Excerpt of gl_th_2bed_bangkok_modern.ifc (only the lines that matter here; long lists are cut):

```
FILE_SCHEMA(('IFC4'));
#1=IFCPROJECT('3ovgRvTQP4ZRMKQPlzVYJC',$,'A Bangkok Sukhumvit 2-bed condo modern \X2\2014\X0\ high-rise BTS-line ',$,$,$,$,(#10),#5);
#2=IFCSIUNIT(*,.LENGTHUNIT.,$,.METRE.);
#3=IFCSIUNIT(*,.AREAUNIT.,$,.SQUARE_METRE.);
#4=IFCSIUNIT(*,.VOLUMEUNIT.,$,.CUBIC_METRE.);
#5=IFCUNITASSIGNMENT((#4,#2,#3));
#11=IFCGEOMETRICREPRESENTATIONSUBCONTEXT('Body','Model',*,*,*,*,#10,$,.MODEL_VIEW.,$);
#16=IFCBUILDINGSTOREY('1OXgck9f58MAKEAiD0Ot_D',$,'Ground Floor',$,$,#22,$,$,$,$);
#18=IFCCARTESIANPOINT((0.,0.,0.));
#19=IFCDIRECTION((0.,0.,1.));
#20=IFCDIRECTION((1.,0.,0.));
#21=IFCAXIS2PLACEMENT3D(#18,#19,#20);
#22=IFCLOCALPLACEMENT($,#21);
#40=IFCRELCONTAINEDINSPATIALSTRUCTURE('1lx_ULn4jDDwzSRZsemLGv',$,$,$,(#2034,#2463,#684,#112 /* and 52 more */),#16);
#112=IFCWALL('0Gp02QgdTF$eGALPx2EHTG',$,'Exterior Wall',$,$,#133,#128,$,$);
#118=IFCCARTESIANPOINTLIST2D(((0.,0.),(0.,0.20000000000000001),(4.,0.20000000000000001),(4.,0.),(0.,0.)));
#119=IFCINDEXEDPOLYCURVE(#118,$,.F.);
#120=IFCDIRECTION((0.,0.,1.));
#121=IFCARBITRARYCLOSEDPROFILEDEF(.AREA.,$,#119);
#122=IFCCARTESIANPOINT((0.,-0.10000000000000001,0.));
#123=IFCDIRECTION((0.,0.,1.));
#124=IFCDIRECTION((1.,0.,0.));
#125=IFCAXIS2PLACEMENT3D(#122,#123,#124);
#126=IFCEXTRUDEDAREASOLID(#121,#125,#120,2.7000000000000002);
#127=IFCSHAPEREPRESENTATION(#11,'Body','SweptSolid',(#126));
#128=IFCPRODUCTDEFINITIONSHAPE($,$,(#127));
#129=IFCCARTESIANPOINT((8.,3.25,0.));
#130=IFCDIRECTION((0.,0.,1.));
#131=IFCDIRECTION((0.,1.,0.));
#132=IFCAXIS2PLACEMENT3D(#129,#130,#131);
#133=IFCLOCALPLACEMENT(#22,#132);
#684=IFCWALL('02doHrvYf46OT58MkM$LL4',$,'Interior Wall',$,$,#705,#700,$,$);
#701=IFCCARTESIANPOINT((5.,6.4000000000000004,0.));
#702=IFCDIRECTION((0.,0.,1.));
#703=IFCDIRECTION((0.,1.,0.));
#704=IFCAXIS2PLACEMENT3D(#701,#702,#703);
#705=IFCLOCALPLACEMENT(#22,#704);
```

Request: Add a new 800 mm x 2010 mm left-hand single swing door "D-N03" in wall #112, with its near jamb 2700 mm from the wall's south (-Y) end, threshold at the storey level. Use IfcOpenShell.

```python
import numpy as np
import ifcopenshell
import ifcopenshell.api.feature
import ifcopenshell.api.geometry
import ifcopenshell.api.root
import ifcopenshell.api.spatial
import ifcopenshell.geom
import ifcopenshell.util.element
import ifcopenshell.util.placement
import ifcopenshell.util.representation
import ifcopenshell.util.shape
import ifcopenshell.util.unit

model = ifcopenshell.open("gl_th_2bed_bangkok_modern.ifc")
unit_scale = ifcopenshell.util.unit.calculate_unit_scale(model)
settings = ifcopenshell.geom.settings()


def volume(element):
    """Net volume in cubic metres, openings subtracted."""
    shape = ifcopenshell.geom.create_shape(settings, element)
    return ifcopenshell.util.shape.get_volume(shape.geometry)


wall = model.by_guid("0Gp02QgdTF$eGALPx2EHTG")
storey = ifcopenshell.util.element.get_container(wall, ifc_class="IfcBuildingStorey")
context = ifcopenshell.util.representation.get_context(model, "Model", "Body", "MODEL_VIEW")
before = volume(wall)

width, height, from_end, sill = 0.8, 2.01, 2.7, 0.0  # metres

# The wall runs along its own X axis, and the end named is its -X end.
wall_shape = ifcopenshell.geom.create_shape(settings, wall)
x, y, z = ifcopenshell.util.shape.get_vertices(wall_shape.geometry).T
start = x.min() + from_end
face, thickness = float(y.min()), float(y.max() - y.min())
wall_matrix = ifcopenshell.util.placement.get_local_placement(wall.ObjectPlacement)
level = ifcopenshell.util.placement.get_local_placement(storey.ObjectPlacement)[2, 3]


def in_wall(x, y):
    """Placement at x, y metres in the wall's axes, at sill height."""
    matrix = wall_matrix.copy()
    matrix[:, 3] = wall_matrix @ np.array([x / unit_scale, y / unit_scale, 0.0, 1.0])
    matrix[2, 3] = level + sill / unit_scale
    return matrix


# Opening: a box that overshoots both wall faces by 50 mm.
opening = ifcopenshell.api.root.create_entity(model, ifc_class="IfcOpeningElement", predefined_type="OPENING")
box = ifcopenshell.api.geometry.add_wall_representation(
    model, context=context, length=width, height=height, thickness=thickness + 0.1
)
ifcopenshell.api.geometry.assign_representation(model, product=opening, representation=box)
ifcopenshell.api.geometry.edit_object_placement(model, product=opening, matrix=in_wall(start, face - 0.05), is_si=False)
ifcopenshell.api.feature.add_feature(model, feature=opening, element=wall)

door = ifcopenshell.api.root.create_entity(model, ifc_class="IfcDoor", name="D-N03", predefined_type="DOOR")
door.OverallWidth, door.OverallHeight = width / unit_scale, height / unit_scale
door.OperationType = "SINGLE_SWING_LEFT"
body = ifcopenshell.api.geometry.add_door_representation(
    model,
    context=context,
    overall_width=door.OverallWidth,
    overall_height=door.OverallHeight,
    operation_type="SINGLE_SWING_LEFT",
    lining_properties={"LiningDepth": thickness / unit_scale, "ThresholdDepth": thickness / unit_scale},
)
ifcopenshell.api.geometry.assign_representation(model, product=door, representation=body)
ifcopenshell.api.spatial.assign_container(model, products=[door], relating_structure=storey)
ifcopenshell.api.feature.add_filling(model, opening=opening, element=door)

# The lining spans the wall, so the door starts at the wall face.
ifcopenshell.api.geometry.edit_object_placement(model, product=door, matrix=in_wall(start, face), is_si=False)

after = volume(wall)

print(f"wall volume {before:.3f} -> {after:.3f} m3")

model.write("gl_th_2bed_bangkok_modern_edited.ifc")
```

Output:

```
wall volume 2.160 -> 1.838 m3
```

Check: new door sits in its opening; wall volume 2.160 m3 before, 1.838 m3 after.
